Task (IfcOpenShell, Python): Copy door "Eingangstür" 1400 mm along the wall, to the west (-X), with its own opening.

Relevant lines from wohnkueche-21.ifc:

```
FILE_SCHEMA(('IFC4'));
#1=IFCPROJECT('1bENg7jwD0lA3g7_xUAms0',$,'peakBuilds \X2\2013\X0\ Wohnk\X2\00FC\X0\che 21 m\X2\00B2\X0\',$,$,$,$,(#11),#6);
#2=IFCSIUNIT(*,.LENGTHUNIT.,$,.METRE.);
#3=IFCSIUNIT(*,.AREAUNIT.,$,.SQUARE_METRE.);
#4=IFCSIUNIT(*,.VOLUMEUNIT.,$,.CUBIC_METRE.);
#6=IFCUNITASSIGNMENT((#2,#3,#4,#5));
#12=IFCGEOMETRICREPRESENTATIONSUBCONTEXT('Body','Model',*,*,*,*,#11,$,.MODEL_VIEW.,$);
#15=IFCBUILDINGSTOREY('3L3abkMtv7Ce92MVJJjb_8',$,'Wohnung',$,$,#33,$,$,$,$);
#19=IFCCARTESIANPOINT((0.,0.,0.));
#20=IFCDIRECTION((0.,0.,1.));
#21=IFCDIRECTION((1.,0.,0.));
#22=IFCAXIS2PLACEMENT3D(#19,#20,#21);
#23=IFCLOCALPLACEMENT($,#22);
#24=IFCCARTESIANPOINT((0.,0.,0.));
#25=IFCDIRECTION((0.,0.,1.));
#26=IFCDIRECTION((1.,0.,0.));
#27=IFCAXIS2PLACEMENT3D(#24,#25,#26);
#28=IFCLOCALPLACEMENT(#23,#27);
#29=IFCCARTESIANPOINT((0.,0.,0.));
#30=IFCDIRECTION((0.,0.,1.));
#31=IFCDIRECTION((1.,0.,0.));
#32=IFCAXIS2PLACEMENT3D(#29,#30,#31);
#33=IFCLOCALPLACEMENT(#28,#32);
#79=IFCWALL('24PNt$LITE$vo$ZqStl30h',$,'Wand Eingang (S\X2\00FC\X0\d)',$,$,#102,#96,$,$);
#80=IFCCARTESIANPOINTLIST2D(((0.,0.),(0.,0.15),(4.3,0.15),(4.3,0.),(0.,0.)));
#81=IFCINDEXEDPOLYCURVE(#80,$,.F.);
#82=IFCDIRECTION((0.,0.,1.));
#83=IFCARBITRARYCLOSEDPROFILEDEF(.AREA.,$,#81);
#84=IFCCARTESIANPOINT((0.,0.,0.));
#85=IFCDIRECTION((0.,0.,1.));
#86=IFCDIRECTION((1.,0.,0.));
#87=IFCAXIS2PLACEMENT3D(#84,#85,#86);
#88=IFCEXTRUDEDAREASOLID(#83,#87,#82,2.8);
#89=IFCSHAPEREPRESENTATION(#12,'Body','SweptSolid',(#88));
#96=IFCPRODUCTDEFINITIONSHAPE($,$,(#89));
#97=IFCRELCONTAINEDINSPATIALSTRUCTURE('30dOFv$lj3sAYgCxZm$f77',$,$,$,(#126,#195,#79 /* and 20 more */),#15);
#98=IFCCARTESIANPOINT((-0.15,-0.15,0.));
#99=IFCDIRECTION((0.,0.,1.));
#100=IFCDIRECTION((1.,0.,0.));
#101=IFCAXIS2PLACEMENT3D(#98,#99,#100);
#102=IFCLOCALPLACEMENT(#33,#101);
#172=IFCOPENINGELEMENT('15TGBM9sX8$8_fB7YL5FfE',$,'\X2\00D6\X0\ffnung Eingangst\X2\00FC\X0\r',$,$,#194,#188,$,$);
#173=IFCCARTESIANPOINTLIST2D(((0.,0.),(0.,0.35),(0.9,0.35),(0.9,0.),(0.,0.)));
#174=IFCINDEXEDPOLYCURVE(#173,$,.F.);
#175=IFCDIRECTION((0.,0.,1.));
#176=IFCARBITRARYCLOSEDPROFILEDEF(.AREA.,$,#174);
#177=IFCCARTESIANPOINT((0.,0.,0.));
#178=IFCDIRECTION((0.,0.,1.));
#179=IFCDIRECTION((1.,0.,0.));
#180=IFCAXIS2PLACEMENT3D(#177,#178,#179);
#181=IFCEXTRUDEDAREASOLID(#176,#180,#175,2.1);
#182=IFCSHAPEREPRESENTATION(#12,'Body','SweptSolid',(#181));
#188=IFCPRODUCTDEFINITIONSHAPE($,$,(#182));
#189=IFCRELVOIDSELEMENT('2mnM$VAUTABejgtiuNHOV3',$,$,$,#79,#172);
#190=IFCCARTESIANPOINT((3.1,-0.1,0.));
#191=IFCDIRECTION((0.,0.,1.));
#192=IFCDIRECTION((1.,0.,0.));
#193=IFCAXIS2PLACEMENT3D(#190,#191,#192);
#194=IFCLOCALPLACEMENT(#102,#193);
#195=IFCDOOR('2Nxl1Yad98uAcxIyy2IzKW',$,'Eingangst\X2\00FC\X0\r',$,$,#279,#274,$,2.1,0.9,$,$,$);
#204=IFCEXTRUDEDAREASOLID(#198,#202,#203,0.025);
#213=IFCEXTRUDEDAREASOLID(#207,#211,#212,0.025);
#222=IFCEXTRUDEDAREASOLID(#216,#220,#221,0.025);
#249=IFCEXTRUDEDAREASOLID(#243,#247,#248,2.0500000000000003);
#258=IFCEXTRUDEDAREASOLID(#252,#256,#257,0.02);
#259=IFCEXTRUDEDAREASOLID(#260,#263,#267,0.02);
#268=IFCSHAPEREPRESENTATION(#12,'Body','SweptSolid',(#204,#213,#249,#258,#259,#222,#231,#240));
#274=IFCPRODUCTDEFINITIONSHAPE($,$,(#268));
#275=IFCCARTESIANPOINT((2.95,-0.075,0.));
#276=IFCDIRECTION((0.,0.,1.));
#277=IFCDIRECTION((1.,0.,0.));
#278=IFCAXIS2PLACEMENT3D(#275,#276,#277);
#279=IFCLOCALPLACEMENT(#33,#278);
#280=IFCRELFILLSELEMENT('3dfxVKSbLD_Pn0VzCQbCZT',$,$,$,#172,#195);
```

```python
import ifcopenshell
import ifcopenshell.api.feature
import ifcopenshell.api.geometry
import ifcopenshell.api.root
import ifcopenshell.geom
import ifcopenshell.util.element
import ifcopenshell.util.placement
import ifcopenshell.util.shape
import ifcopenshell.util.unit

model = ifcopenshell.open("wohnkueche-21.ifc")
unit_scale = ifcopenshell.util.unit.calculate_unit_scale(model)
settings = ifcopenshell.geom.settings()


def volume(element):
    """Net volume in cubic metres, openings subtracted."""
    shape = ifcopenshell.geom.create_shape(settings, element)
    return ifcopenshell.util.shape.get_volume(shape.geometry)


door = model.by_id(195)
opening = door.FillsVoids[0].RelatingOpeningElement
wall = opening.VoidsElements[0].RelatingBuildingElement
before = volume(wall)
shift = ifcopenshell.util.placement.get_local_placement(wall.ObjectPlacement)[:3, 0] * -1.4 / unit_scale

# copy_class copies the void relationship, type, container and properties, but no geometry.
new_opening = ifcopenshell.api.root.copy_class(model, product=opening)
new_opening.Representation = ifcopenshell.util.element.copy_deep(
    model, opening.Representation, exclude=["IfcGeometricRepresentationContext", "IfcRepresentationMap"]
)
new_door = ifcopenshell.api.root.copy_class(model, product=door)
new_door.Representation = ifcopenshell.util.element.copy_deep(
    model, door.Representation, exclude=["IfcGeometricRepresentationContext", "IfcRepresentationMap"]
)
ifcopenshell.api.feature.add_filling(model, opening=new_opening, element=new_door)

for old, new in ((opening, new_opening), (door, new_door)):
    matrix = ifcopenshell.util.placement.get_local_placement(old.ObjectPlacement)
    matrix[:3, 3] += shift
    ifcopenshell.api.geometry.edit_object_placement(model, product=new, matrix=matrix, is_si=False)

after = volume(wall)

print(f"wall volume {before:.3f} -> {after:.3f} m3")

model.write("wohnkueche-21-out.ifc")
```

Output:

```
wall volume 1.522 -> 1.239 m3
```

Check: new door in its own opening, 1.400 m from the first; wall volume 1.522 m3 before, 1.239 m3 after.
